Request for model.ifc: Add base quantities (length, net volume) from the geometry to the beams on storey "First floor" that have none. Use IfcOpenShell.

First a look at what the model holds.

```python
import ifcopenshell
import ifcopenshell.util.element
import ifcopenshell.util.unit

model = ifcopenshell.open("model.ifc")
print(model.schema)
for unit_type in ("LENGTHUNIT", "AREAUNIT", "VOLUMEUNIT"):
    print(unit_type, ifcopenshell.util.unit.calculate_unit_scale(model, unit_type))
storey = next(s for s in model.by_type("IfcBuildingStorey") if s.Name == "First floor")
beams = [e for e in ifcopenshell.util.element.get_decomposition(storey) if e.is_a("IfcBeam")]
for e in sorted(beams, key=lambda e: e.id()):
    print(e.id(), e.is_a(), e.Name, list(ifcopenshell.util.element.get_psets(e, qtos_only=True)), sep=" | ")
```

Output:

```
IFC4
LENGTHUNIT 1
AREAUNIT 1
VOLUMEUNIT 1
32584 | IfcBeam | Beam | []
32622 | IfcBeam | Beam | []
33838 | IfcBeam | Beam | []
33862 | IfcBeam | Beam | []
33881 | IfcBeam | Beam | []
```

```python
import ifcopenshell
import ifcopenshell.api.pset
import ifcopenshell.geom
import ifcopenshell.util.element
import ifcopenshell.util.shape
import ifcopenshell.util.unit

model = ifcopenshell.open("model.ifc")
unit_scale = ifcopenshell.util.unit.calculate_unit_scale(model)
volume_scale = ifcopenshell.util.unit.calculate_unit_scale(model, "VOLUMEUNIT")
settings = ifcopenshell.geom.settings()

storey = next(s for s in model.by_type("IfcBuildingStorey") if s.Name == "First floor")
beams = [e for e in ifcopenshell.util.element.get_decomposition(storey) if e.is_a("IfcBeam")]

for e in sorted(beams, key=lambda e: e.id()):
    if ifcopenshell.util.element.get_psets(e, qtos_only=True, should_inherit=False):
        continue
    # Geometry comes back in metres, in the element's own axes.
    shape = ifcopenshell.geom.create_shape(settings, e)
    values = {
        "Length": ifcopenshell.util.shape.get_max_xyz(shape.geometry) / unit_scale,
        "NetVolume": ifcopenshell.util.shape.get_volume(shape.geometry) / volume_scale,
    }
    qto = ifcopenshell.api.pset.add_qto(model, product=e, name="Qto_BeamBaseQuantities")
    ifcopenshell.api.pset.edit_qto(model, qto=qto, properties=values)
    print(e.id(), {k: round(v, 3) for k, v in values.items()})

model.write("model_rev.ifc")
```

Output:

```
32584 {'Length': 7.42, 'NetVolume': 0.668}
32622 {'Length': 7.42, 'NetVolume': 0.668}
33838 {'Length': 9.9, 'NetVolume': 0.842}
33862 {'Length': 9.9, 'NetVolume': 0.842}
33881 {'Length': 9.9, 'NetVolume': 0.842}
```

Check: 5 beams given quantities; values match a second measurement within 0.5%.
